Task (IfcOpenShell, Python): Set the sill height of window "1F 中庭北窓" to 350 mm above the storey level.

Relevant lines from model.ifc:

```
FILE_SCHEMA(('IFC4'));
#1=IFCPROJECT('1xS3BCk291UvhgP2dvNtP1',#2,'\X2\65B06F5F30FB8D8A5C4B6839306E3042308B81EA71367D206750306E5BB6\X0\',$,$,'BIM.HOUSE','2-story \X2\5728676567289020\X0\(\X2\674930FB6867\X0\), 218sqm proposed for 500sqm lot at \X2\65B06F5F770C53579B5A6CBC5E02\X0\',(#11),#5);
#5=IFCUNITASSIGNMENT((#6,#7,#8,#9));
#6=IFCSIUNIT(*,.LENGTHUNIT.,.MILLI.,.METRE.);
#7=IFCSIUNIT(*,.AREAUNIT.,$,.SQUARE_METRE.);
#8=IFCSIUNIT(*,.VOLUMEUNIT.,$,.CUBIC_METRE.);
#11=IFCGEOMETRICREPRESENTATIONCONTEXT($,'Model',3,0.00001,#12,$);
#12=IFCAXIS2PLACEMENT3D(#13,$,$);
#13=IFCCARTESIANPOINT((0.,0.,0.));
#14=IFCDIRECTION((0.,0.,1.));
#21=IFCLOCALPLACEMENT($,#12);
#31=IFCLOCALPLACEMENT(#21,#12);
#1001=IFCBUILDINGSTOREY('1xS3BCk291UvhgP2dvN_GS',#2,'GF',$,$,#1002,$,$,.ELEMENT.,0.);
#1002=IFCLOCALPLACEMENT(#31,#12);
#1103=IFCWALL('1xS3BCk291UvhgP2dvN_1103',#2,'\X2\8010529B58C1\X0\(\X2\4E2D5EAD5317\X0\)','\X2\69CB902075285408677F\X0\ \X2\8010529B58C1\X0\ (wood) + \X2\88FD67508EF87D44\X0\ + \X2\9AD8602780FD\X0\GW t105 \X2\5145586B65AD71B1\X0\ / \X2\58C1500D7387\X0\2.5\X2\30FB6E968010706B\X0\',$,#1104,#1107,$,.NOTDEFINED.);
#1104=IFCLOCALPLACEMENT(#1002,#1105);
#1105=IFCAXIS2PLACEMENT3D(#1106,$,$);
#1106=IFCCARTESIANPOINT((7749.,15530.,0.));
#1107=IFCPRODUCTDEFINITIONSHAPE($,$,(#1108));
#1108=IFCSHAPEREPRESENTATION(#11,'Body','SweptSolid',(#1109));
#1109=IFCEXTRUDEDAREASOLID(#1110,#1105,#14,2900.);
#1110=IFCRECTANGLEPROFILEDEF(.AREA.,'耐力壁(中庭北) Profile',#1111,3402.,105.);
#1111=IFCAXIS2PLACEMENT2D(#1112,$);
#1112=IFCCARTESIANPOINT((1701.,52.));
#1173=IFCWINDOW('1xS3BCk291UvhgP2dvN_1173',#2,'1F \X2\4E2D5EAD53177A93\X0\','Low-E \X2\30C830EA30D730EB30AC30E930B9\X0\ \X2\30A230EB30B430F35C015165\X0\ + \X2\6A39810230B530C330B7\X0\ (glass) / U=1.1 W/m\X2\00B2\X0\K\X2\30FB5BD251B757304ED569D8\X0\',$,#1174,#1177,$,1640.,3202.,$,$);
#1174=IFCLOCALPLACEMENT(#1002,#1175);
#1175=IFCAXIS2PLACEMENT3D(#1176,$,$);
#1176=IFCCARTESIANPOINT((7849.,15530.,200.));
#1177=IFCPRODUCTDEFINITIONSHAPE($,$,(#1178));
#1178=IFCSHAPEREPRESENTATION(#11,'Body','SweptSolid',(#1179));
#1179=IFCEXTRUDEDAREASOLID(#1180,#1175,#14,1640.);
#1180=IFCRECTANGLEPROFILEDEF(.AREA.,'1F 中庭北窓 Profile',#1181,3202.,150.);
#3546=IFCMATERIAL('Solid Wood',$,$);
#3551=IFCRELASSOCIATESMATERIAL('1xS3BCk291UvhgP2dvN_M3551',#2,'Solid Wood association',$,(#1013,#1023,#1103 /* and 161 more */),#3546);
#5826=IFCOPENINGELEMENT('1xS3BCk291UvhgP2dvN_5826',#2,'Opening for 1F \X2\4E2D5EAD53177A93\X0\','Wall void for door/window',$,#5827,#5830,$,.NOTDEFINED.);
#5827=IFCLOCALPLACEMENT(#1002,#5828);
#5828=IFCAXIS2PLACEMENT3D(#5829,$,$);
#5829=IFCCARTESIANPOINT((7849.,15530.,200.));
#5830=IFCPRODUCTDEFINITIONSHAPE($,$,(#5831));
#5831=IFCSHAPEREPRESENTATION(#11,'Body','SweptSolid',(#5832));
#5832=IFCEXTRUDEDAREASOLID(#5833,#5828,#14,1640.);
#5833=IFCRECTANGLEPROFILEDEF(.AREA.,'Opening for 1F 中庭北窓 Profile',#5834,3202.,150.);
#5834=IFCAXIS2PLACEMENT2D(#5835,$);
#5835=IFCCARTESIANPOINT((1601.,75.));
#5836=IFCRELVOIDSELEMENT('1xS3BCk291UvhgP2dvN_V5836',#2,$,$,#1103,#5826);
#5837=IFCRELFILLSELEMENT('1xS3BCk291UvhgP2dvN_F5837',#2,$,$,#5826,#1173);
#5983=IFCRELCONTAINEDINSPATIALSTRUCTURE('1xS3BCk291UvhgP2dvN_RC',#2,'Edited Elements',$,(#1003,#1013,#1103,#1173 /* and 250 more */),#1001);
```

```python
import numpy as np
import ifcopenshell
import ifcopenshell.api.geometry
import ifcopenshell.geom
import ifcopenshell.util.element
import ifcopenshell.util.placement
import ifcopenshell.util.shape
import ifcopenshell.util.unit

model = ifcopenshell.open("model.ifc")
unit_scale = ifcopenshell.util.unit.calculate_unit_scale(model)

window = model.by_guid("1xS3BCk291UvhgP2dvN_1173")
opening = window.FillsVoids[0].RelatingOpeningElement
storey = ifcopenshell.util.element.get_container(window, ifc_class="IfcBuildingStorey")
level = ifcopenshell.util.placement.get_local_placement(storey.ObjectPlacement)[2, 3]

# The opening's origin need not be at the sill, so measure its lowest point.
shape = ifcopenshell.geom.create_shape(ifcopenshell.geom.settings(), opening)
bottom = ifcopenshell.util.shape.get_shape_bottom_elevation(shape, shape.geometry) / unit_scale
dz = level + 350.0 - bottom

shift = np.array([0.0, 0.0, dz])
# The window is not placed relative to its opening, so move both.
for product in (opening, window):
    matrix = ifcopenshell.util.placement.get_local_placement(product.ObjectPlacement)
    matrix[:3, 3] += shift
    ifcopenshell.api.geometry.edit_object_placement(model, product=product, matrix=matrix, is_si=False)

print(f"moved by {dz * unit_scale:+.3f} m")

model.write("model_updated.ifc")
```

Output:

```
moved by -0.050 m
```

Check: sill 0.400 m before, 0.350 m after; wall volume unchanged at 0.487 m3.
